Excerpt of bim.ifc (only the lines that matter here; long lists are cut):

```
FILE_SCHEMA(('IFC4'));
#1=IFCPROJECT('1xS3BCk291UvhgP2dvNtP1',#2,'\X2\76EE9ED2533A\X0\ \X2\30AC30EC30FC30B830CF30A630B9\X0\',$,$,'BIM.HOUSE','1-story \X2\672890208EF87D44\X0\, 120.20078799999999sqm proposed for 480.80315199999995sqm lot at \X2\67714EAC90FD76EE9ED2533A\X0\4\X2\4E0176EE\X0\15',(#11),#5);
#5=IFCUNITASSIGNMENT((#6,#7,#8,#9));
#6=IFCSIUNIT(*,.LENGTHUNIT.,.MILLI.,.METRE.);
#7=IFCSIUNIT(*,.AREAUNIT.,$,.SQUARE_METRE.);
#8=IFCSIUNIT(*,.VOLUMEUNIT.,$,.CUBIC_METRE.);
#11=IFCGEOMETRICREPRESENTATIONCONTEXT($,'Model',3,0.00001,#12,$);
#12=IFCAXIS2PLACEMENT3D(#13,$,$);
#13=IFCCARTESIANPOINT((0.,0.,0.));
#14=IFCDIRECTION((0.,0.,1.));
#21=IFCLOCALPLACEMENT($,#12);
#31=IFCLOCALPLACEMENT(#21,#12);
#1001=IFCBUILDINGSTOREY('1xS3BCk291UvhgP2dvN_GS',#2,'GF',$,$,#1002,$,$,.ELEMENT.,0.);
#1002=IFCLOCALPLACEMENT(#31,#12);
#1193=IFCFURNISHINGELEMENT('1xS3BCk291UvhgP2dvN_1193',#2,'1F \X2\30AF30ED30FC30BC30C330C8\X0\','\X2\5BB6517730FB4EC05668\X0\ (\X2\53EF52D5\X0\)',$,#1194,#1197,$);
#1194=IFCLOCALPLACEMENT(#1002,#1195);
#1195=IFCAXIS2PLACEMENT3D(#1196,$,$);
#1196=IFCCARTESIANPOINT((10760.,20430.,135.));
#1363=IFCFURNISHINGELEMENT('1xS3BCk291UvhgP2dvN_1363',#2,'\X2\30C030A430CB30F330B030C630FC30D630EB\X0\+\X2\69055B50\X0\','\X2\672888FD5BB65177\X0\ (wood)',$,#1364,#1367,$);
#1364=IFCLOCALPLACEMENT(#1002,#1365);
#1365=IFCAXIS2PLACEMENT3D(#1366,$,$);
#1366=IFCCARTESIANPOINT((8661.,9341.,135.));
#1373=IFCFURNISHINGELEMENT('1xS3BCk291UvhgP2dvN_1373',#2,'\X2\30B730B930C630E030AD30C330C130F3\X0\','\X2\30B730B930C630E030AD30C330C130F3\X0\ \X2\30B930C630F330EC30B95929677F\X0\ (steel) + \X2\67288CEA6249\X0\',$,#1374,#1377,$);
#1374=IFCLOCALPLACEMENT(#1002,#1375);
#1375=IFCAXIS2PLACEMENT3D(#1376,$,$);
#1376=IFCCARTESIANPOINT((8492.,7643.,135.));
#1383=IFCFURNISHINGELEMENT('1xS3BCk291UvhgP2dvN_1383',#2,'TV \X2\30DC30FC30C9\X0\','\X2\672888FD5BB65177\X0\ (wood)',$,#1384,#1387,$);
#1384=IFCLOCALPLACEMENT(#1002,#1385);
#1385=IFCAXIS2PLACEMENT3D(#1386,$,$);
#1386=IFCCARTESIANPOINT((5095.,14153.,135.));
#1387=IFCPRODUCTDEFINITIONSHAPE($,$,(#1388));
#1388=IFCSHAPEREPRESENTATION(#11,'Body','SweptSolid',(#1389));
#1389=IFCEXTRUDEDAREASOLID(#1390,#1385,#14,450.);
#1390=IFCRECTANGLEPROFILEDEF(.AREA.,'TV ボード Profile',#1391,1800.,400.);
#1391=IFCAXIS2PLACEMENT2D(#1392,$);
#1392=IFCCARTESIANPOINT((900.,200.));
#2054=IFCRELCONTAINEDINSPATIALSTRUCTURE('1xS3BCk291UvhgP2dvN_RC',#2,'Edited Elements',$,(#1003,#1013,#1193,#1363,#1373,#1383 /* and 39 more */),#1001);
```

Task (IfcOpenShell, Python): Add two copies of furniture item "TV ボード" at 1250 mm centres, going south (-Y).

```python
import numpy as np
import ifcopenshell
import ifcopenshell.api.geometry
import ifcopenshell.api.root
import ifcopenshell.util.element
import ifcopenshell.util.placement

model = ifcopenshell.open("bim.ifc")


def reuse_history(source, copy):
    """copy_class also copies each property set's owner history, people and application; keep the originals."""
    for rel in copy.IsDefinedBy:
        if rel.is_a("IfcRelDefinesByProperties") and (history := rel.RelatingPropertyDefinition.OwnerHistory):
            rel.RelatingPropertyDefinition.OwnerHistory = source.OwnerHistory
            ifcopenshell.util.element.remove_deep2(model, history)


source = model.by_guid("1xS3BCk291UvhgP2dvN_1383")
base = ifcopenshell.util.placement.get_local_placement(source.ObjectPlacement)
step = np.array([0.0, -1.0, 0.0]) * 1250.0

for i in range(1, 3):
    copy = ifcopenshell.api.root.copy_class(model, product=source)
    copy.Representation = ifcopenshell.util.element.copy_deep(
        model, source.Representation, exclude=["IfcGeometricRepresentationContext", "IfcRepresentationMap"]
    )
    reuse_history(source, copy)
    matrix = base.copy()
    matrix[:3, 3] += i * step
    print("added at", matrix[:3, 3].round(3) + 0.0)
    ifcopenshell.api.geometry.edit_object_placement(model, product=copy, matrix=matrix, is_si=False)

model.write("bim_edited.ifc")
```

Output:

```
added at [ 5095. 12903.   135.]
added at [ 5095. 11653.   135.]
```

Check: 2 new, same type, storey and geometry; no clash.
